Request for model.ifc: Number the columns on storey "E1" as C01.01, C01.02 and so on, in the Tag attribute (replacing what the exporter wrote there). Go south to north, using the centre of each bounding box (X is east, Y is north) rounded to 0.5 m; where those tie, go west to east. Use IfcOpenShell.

First a look at what the model holds.

```python
import ifcopenshell
import ifcopenshell.util.element
import ifcopenshell.util.placement

model = ifcopenshell.open("model.ifc")
print(model.schema)
storey = next(s for s in model.by_type("IfcBuildingStorey") if s.Name == "E1")
columns = [e for e in ifcopenshell.util.element.get_decomposition(storey) if e.is_a("IfcColumn")]
for e in sorted(columns, key=lambda e: e.id()):
    origin = ifcopenshell.util.placement.get_local_placement(e.ObjectPlacement)[:3, 3]
    print(e.id(), e.Tag, e.Name, origin.round(2) + 0.0, sep=" | ")
```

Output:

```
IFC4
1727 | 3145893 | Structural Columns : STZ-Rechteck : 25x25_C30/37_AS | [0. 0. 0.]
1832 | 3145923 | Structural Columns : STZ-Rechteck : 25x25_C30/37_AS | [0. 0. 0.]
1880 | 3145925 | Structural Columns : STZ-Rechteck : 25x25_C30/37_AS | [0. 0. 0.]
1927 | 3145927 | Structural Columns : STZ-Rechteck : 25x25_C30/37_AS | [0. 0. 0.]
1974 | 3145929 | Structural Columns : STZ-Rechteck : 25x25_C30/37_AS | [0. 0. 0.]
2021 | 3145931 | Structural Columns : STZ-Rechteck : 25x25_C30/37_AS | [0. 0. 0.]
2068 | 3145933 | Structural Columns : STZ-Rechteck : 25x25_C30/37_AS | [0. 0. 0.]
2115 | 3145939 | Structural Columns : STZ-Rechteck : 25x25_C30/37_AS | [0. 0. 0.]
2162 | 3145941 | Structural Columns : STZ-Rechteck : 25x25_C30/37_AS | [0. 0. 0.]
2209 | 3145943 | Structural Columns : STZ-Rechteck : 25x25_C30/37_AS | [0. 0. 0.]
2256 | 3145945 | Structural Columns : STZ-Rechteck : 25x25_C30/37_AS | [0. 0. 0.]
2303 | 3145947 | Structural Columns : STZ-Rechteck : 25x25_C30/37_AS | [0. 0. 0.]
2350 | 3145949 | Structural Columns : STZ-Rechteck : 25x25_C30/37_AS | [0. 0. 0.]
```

```python
import ifcopenshell
import ifcopenshell.geom
import ifcopenshell.util.element
import ifcopenshell.util.shape

model = ifcopenshell.open("model.ifc")
settings = ifcopenshell.geom.settings()
settings.set("use-world-coords", True)


def centre(element):
    shape = ifcopenshell.geom.create_shape(settings, element)
    return ifcopenshell.util.shape.get_bbox_centroid(shape.geometry)


storey = next(s for s in model.by_type("IfcBuildingStorey") if s.Name == "E1")
columns = [e for e in ifcopenshell.util.element.get_decomposition(storey) if e.is_a("IfcColumn")]

# Insertion points can sit at a corner or the storey origin, so sort by the geometry (in metres).
centres = {e: centre(e) for e in columns}
columns.sort(key=lambda e: (round(centres[e][1] / 0.5), centres[e][0]))

for i, e in enumerate(columns, start=1):
    number = f"C01.{i:02d}"
    e.Tag = number
    print(e.id(), number)

model.write("model_edited.ifc")
```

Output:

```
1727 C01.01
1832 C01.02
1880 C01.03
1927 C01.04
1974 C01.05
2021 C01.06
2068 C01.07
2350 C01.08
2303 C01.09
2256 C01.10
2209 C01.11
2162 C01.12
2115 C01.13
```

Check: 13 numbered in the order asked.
